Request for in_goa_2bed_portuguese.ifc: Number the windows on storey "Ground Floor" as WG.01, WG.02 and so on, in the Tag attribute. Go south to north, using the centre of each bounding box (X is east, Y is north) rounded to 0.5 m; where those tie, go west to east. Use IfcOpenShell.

First a look at what the model holds.

```python
import ifcopenshell
import ifcopenshell.util.element
import ifcopenshell.util.placement

model = ifcopenshell.open("in_goa_2bed_portuguese.ifc")
print(model.schema)
storey = next(s for s in model.by_type("IfcBuildingStorey") if s.Name == "Ground Floor")
windows = [e for e in ifcopenshell.util.element.get_decomposition(storey) if e.is_a("IfcWindow")]
for e in sorted(windows, key=lambda e: e.id()):
    origin = ifcopenshell.util.placement.get_local_placement(e.ObjectPlacement)[:3, 3]
    print(e.id(), e.Tag, e.Name, origin.round(2) + 0.0, sep=" | ")
```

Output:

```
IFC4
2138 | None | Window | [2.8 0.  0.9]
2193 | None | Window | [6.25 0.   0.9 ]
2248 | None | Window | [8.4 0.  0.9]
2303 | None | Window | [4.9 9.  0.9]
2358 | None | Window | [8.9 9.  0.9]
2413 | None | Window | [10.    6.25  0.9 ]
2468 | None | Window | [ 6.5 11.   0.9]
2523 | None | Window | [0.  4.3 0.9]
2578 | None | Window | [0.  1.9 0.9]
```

```python
import ifcopenshell
import ifcopenshell.geom
import ifcopenshell.util.element
import ifcopenshell.util.shape

model = ifcopenshell.open("in_goa_2bed_portuguese.ifc")
settings = ifcopenshell.geom.settings()
settings.set("use-world-coords", True)


def centre(element):
    shape = ifcopenshell.geom.create_shape(settings, element)
    return ifcopenshell.util.shape.get_bbox_centroid(shape.geometry)


storey = next(s for s in model.by_type("IfcBuildingStorey") if s.Name == "Ground Floor")
windows = [e for e in ifcopenshell.util.element.get_decomposition(storey) if e.is_a("IfcWindow")]

# Insertion points can sit at a corner or the storey origin, so sort by the geometry (in metres).
centres = {e: centre(e) for e in windows}
windows.sort(key=lambda e: (round(centres[e][1] / 0.5), centres[e][0]))

for i, e in enumerate(windows, start=1):
    number = f"WG.{i:02d}"
    e.Tag = number
    print(e.id(), number)

model.write("in_goa_2bed_portuguese_rev.ifc")
```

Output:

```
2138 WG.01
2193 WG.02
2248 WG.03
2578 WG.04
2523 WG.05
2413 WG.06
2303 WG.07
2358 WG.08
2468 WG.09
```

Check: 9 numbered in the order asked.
